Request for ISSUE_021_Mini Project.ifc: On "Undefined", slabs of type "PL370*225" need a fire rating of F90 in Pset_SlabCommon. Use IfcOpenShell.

First a look at what the model holds.

```python
import ifcopenshell
import ifcopenshell.util.element

model = ifcopenshell.open("ISSUE_021_Mini Project.ifc")
print(model.schema)
storey = next(s for s in model.by_type("IfcBuildingStorey") if s.Name == "Undefined")
slabs = [e for e in ifcopenshell.util.element.get_decomposition(storey) if e.is_a("IfcSlab")]
seen = {}
for e in slabs:
    element_type = ifcopenshell.util.element.get_type(e)
    key = (element_type.Name if element_type != e and element_type else None, ifcopenshell.util.element.get_pset(e, "Pset_SlabCommon", "FireRating"))
    seen[key] = seen.get(key, 0) + 1
for (name, value), count in sorted(seen.items(), key=str):
    print(count, "x", name, "|", value)
```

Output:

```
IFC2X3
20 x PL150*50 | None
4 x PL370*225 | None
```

```python
import ifcopenshell
import ifcopenshell.api.pset
import ifcopenshell.util.element

model = ifcopenshell.open("ISSUE_021_Mini Project.ifc")

storey = next(s for s in model.by_type("IfcBuildingStorey") if s.Name == "Undefined")
slabs = [e for e in ifcopenshell.util.element.get_decomposition(storey) if e.is_a("IfcSlab")]

count = 0
for e in slabs:
    element_type = ifcopenshell.util.element.get_type(e)
    if element_type in (None, e) or element_type.Name != "PL370*225":
        continue
    found = ifcopenshell.util.element.get_pset(e, "Pset_SlabCommon", should_inherit=False)
    if found:
        pset = model.by_id(found["id"])
        if len(ifcopenshell.util.element.get_elements_by_pset(pset)) > 1:
            pset = ifcopenshell.api.pset.unshare_pset(model, products=[e], pset=pset)[0]
    else:
        pset = ifcopenshell.api.pset.add_pset(model, product=e, name="Pset_SlabCommon")
    ifcopenshell.api.pset.edit_pset(model, pset=pset, properties={"FireRating": "F90"})
    count += 1

print(count, "slabs updated")

model.write("ISSUE_021_Mini Project-out.ifc")
```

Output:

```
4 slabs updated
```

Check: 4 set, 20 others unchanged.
